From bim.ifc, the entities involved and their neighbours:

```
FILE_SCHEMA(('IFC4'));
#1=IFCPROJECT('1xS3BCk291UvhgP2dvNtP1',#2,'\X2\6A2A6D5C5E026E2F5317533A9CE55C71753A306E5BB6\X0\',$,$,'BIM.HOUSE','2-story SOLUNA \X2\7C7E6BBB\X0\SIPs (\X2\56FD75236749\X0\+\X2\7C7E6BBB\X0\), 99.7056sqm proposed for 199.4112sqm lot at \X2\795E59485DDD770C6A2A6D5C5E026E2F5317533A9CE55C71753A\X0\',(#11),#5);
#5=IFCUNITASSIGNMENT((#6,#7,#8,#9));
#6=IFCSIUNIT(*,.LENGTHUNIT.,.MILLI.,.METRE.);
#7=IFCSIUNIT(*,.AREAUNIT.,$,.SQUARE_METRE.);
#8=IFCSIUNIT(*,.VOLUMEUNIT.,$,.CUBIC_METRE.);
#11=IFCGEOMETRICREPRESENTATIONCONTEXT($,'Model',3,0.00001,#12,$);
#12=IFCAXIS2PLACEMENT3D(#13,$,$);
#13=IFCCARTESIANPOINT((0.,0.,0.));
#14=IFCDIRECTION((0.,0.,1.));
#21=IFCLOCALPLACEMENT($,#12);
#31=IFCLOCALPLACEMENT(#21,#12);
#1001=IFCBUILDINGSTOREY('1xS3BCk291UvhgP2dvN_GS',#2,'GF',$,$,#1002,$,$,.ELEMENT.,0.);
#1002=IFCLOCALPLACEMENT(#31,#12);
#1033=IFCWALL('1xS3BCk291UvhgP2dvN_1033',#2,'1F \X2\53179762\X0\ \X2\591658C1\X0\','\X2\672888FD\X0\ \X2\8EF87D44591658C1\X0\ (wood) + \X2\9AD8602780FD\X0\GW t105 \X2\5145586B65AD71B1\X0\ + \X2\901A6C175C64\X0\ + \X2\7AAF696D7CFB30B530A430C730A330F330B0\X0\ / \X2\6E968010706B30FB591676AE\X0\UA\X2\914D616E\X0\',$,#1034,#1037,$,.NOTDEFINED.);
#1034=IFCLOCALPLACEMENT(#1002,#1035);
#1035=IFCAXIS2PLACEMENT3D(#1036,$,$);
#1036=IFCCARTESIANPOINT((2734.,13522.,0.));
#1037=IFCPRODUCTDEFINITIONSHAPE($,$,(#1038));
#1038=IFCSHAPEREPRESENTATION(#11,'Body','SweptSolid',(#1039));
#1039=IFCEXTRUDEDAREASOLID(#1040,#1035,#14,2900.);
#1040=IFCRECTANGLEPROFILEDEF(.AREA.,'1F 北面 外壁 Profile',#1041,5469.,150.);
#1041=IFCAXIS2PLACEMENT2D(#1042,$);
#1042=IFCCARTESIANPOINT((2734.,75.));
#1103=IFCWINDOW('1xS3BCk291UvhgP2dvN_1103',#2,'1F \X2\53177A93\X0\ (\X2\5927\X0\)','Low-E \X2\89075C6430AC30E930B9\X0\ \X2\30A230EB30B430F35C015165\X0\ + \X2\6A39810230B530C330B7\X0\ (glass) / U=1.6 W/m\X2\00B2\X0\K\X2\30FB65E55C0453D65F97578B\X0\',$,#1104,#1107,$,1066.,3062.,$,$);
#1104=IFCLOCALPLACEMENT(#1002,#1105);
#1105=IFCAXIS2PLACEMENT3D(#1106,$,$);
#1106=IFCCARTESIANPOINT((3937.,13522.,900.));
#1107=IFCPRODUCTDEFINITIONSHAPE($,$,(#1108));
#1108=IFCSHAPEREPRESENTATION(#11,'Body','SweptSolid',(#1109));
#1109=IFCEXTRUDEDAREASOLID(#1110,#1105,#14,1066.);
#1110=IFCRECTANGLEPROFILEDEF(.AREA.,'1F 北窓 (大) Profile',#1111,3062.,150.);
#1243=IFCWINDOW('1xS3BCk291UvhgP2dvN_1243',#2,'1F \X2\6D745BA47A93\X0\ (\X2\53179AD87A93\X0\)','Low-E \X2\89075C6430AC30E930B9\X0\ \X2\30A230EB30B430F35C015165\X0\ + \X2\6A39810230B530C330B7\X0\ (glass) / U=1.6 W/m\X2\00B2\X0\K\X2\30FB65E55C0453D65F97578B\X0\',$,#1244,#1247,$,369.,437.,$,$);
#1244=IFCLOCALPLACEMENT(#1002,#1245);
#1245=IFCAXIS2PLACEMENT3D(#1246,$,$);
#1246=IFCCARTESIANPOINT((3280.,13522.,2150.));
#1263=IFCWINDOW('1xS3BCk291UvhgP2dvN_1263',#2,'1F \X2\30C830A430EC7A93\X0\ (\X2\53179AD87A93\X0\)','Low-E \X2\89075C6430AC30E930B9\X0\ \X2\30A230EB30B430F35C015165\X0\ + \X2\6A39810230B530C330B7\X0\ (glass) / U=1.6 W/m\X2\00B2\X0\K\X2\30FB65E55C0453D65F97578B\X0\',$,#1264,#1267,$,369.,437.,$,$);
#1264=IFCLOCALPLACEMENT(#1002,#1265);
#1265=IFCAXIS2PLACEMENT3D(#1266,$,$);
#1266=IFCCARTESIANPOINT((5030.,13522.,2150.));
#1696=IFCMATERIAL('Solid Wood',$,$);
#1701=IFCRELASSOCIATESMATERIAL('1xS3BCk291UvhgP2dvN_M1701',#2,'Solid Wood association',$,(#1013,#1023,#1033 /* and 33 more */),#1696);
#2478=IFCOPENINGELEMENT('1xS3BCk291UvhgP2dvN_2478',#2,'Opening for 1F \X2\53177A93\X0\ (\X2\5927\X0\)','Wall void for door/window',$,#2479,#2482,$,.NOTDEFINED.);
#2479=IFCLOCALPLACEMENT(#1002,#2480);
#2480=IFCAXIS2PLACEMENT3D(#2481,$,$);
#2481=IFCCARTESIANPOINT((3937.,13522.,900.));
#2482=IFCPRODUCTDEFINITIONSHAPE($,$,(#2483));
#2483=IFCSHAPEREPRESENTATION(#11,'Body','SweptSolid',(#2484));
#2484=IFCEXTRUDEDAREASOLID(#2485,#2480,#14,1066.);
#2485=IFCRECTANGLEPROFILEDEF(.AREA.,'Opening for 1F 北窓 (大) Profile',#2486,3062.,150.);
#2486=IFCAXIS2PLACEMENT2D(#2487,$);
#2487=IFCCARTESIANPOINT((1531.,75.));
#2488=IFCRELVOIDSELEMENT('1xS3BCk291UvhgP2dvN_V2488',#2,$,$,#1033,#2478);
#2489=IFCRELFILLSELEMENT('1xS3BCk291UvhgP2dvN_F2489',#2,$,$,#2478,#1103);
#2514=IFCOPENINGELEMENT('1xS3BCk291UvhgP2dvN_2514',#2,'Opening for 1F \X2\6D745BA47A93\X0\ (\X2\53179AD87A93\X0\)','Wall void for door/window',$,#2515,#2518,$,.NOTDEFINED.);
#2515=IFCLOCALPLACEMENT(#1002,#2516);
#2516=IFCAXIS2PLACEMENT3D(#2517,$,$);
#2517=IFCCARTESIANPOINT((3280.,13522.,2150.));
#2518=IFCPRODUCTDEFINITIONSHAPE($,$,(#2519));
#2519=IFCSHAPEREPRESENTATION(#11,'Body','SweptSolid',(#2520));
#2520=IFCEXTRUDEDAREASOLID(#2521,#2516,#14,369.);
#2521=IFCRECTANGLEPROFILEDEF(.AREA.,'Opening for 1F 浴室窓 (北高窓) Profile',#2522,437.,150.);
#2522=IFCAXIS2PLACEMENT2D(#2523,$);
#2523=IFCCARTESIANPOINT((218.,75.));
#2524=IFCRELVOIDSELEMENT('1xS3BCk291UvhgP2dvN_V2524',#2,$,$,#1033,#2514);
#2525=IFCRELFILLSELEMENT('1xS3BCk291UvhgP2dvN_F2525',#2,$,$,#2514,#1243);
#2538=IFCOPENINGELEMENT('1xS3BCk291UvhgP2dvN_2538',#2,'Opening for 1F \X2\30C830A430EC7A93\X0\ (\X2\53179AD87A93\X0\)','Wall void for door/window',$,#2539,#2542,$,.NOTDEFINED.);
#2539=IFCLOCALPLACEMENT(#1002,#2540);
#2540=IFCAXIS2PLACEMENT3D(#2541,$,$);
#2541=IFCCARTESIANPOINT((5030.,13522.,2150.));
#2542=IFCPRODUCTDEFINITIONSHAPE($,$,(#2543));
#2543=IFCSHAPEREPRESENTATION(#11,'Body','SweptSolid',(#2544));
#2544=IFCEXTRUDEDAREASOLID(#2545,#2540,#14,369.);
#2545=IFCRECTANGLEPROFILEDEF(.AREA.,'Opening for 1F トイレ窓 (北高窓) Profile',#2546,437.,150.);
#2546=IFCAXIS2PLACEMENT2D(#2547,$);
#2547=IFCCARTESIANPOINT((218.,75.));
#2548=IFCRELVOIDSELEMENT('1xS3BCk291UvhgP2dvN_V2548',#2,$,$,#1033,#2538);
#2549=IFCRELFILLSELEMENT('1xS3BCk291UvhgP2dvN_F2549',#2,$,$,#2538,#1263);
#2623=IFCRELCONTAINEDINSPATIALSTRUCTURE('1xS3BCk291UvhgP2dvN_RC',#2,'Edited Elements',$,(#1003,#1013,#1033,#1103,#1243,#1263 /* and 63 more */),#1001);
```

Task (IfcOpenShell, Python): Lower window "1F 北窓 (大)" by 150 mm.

```python
import numpy as np
import ifcopenshell
import ifcopenshell.api.geometry
import ifcopenshell.util.placement
import ifcopenshell.util.unit

model = ifcopenshell.open("bim.ifc")
unit_scale = ifcopenshell.util.unit.calculate_unit_scale(model)

window = model.by_id(1103)
opening = window.FillsVoids[0].RelatingOpeningElement
dz = -0.15 / unit_scale

shift = np.array([0.0, 0.0, dz])
# The window is not placed relative to its opening, so move both.
for product in (opening, window):
    matrix = ifcopenshell.util.placement.get_local_placement(product.ObjectPlacement)
    matrix[:3, 3] += shift
    ifcopenshell.api.geometry.edit_object_placement(model, product=product, matrix=matrix, is_si=False)

print(f"moved by {dz * unit_scale:+.3f} m")

model.write("bim_rev.ifc")
```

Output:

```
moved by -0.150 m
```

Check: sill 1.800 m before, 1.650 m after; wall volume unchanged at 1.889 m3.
